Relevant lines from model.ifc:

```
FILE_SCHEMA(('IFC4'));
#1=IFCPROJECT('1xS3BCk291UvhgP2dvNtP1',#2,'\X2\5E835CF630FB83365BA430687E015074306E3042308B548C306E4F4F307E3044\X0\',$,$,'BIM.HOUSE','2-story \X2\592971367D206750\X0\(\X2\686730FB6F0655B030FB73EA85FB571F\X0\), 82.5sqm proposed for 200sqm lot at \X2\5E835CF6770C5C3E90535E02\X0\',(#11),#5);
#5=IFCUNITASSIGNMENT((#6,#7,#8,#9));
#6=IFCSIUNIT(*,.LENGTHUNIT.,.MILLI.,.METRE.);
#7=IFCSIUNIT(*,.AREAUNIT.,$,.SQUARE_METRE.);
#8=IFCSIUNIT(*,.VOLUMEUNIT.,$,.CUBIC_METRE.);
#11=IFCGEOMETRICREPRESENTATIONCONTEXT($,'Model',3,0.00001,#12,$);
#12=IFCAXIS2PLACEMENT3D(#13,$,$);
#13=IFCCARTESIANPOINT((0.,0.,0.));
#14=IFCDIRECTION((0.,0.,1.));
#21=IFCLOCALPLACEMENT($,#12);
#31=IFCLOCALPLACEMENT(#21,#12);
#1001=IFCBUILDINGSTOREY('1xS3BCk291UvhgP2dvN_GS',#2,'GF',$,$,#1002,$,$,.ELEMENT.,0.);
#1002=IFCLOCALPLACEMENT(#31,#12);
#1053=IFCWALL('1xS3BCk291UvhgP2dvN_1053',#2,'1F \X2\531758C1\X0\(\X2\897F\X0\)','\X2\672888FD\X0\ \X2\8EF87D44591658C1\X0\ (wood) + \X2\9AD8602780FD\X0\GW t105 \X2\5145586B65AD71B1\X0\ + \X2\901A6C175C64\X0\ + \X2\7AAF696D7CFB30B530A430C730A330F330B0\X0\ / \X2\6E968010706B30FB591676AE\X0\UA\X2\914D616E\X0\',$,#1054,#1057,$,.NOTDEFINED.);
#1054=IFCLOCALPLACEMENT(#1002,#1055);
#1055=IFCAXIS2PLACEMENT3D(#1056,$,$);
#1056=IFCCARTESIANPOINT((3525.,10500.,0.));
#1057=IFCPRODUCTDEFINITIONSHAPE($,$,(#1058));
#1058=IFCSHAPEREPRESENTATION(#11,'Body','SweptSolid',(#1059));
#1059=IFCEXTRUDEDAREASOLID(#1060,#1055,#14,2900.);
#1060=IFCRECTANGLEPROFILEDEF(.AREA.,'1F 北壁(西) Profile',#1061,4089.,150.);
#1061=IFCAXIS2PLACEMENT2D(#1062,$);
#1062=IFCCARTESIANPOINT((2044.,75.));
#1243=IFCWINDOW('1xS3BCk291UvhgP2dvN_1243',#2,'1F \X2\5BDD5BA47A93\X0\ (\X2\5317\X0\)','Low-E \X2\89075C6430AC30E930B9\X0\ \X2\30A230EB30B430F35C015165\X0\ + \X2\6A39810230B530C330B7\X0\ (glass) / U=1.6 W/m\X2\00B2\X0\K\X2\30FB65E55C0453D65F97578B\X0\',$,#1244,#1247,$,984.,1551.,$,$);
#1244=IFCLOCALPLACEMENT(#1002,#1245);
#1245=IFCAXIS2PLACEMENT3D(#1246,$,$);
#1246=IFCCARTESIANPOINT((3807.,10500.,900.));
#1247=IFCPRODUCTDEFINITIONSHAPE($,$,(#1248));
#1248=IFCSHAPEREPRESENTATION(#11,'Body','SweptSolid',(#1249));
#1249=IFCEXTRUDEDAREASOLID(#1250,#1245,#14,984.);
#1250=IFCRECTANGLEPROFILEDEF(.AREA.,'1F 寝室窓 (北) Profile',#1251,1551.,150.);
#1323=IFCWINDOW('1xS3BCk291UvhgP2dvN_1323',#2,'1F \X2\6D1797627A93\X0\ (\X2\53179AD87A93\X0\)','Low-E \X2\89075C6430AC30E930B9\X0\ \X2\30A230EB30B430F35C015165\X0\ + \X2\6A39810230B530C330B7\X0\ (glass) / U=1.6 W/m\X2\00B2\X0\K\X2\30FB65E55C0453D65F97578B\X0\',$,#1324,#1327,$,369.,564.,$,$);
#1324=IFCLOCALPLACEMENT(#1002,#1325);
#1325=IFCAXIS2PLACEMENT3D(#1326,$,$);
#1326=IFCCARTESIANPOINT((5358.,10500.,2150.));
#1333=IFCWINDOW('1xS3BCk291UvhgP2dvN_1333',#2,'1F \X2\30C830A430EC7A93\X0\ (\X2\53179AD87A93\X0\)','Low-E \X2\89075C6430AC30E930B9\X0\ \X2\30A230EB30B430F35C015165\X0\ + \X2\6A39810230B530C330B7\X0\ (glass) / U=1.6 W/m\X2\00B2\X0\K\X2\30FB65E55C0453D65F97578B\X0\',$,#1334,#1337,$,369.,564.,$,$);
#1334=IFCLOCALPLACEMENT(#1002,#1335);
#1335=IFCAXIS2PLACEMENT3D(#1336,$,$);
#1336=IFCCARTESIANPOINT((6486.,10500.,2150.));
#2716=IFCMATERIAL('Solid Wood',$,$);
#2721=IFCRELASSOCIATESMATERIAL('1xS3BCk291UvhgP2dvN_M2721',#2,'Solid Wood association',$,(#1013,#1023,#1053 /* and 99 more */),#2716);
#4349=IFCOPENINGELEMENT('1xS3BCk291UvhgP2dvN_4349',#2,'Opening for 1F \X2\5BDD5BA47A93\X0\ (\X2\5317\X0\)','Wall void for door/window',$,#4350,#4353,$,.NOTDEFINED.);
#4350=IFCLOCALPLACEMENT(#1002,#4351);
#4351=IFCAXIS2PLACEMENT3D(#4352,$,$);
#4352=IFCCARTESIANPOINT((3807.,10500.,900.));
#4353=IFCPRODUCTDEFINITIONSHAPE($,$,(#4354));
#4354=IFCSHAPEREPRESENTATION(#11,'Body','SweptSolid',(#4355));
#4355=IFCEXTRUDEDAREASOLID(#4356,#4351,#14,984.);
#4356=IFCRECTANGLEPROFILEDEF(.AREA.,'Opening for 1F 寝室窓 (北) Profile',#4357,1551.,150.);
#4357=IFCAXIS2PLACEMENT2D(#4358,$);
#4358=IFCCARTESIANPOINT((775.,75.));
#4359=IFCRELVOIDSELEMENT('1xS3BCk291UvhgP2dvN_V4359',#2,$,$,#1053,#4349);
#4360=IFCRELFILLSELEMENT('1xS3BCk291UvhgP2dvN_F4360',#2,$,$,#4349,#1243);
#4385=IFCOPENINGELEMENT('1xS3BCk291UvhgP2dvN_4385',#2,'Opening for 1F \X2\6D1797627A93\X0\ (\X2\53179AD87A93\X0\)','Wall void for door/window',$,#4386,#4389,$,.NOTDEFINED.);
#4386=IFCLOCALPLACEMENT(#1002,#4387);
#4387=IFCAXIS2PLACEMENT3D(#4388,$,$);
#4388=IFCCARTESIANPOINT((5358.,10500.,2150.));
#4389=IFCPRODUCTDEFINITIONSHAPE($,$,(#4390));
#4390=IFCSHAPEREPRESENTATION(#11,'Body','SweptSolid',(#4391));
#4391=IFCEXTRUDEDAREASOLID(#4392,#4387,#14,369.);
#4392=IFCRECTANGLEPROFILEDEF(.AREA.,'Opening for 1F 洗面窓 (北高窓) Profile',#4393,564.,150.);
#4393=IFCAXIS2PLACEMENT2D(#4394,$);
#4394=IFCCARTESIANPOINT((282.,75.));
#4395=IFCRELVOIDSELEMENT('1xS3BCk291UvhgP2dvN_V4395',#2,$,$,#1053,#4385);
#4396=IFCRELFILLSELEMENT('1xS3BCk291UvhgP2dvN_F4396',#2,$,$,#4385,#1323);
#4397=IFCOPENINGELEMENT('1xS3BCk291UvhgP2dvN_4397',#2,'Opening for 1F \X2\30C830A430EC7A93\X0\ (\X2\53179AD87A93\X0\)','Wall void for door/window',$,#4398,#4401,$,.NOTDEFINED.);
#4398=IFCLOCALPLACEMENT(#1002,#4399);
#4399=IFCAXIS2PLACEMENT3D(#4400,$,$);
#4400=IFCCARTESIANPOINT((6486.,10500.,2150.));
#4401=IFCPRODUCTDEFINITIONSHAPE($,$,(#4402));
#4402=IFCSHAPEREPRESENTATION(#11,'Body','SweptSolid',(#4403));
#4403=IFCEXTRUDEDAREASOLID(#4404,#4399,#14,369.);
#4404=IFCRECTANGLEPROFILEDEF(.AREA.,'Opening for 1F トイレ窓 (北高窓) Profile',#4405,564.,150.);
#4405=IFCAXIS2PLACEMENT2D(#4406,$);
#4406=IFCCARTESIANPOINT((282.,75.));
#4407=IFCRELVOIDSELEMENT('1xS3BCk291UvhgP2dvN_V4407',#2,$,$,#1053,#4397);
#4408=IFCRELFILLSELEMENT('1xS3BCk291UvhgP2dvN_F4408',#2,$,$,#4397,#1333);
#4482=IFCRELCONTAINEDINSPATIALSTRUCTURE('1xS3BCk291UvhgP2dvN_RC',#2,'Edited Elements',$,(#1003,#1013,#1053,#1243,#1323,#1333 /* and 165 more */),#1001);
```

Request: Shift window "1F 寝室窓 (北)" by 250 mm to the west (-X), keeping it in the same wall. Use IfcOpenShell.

```python
import ifcopenshell
import ifcopenshell.api.geometry
import ifcopenshell.util.placement
import ifcopenshell.util.unit

model = ifcopenshell.open("model.ifc")
unit_scale = ifcopenshell.util.unit.calculate_unit_scale(model)

window = model.by_id(1243)
opening = window.FillsVoids[0].RelatingOpeningElement
wall = opening.VoidsElements[0].RelatingBuildingElement

wall_matrix = ifcopenshell.util.placement.get_local_placement(wall.ObjectPlacement)
shift = wall_matrix[:3, 0] * -0.25 / unit_scale
before = ifcopenshell.util.placement.get_local_placement(window.ObjectPlacement)[:3, 3].copy()

# The window is not placed relative to its opening, so move both.
for product in (opening, window):
    matrix = ifcopenshell.util.placement.get_local_placement(product.ObjectPlacement)
    matrix[:3, 3] += shift
    ifcopenshell.api.geometry.edit_object_placement(model, product=product, matrix=matrix, is_si=False)

after = ifcopenshell.util.placement.get_local_placement(window.ObjectPlacement)[:3, 3]
print("window moved by", (after - before).round(3) + 0.0)

model.write("model-out.ifc")
```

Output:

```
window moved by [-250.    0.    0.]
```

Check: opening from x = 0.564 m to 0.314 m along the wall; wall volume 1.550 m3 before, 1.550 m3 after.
